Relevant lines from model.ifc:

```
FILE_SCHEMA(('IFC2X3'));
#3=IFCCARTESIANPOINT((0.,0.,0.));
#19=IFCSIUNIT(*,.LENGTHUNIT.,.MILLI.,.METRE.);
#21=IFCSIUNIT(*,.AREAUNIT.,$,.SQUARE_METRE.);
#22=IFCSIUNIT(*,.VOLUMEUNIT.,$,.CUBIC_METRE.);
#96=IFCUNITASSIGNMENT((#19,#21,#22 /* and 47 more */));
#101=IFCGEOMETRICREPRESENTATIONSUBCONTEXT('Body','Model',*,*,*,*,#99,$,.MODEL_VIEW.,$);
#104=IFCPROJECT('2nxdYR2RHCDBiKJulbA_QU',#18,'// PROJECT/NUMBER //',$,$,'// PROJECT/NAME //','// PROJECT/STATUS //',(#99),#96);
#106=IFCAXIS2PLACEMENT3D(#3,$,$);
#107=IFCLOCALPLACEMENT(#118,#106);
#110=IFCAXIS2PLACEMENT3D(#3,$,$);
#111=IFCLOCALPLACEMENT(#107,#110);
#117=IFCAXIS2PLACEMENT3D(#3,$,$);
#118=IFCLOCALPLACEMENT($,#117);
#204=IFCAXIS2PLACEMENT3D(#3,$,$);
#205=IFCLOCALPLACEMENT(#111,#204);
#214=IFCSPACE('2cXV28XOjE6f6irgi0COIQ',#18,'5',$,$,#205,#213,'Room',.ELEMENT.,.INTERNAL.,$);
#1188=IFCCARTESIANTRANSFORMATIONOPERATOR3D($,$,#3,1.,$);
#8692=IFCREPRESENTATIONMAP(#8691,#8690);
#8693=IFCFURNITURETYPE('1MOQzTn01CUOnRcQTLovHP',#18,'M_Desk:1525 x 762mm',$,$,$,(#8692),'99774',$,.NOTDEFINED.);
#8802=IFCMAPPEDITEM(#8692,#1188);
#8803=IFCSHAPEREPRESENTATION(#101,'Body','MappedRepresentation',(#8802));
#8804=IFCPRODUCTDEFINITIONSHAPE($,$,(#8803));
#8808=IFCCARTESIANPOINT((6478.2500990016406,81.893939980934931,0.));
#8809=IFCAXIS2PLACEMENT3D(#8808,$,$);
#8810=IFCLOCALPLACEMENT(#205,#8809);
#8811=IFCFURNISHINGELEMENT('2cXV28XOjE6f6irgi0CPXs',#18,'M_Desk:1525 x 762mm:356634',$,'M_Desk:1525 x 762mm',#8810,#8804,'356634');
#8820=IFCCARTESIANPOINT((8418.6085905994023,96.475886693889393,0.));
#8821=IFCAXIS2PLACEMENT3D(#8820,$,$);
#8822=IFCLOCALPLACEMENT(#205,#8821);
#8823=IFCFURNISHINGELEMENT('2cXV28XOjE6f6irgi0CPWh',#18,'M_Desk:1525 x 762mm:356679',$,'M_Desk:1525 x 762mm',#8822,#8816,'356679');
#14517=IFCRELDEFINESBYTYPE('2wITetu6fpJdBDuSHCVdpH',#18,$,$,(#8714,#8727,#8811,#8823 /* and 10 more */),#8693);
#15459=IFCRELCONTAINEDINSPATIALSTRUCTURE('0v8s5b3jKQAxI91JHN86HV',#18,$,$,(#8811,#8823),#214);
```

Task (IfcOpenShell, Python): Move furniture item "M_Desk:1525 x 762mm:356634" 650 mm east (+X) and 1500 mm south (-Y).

```python
import ifcopenshell
import ifcopenshell.api.geometry
import ifcopenshell.util.placement
import ifcopenshell.util.unit

model = ifcopenshell.open("model.ifc")
unit_scale = ifcopenshell.util.unit.calculate_unit_scale(model)

item = model.by_guid("2cXV28XOjE6f6irgi0CPXs")
matrix = ifcopenshell.util.placement.get_local_placement(item.ObjectPlacement)
matrix[0, 3] += 0.65 / unit_scale
matrix[1, 3] -= 1.5 / unit_scale
ifcopenshell.api.geometry.edit_object_placement(model, product=item, matrix=matrix, is_si=False)

print(ifcopenshell.util.placement.get_local_placement(item.ObjectPlacement).round(3) + 0.0)

model.write("model_v2.ifc")
```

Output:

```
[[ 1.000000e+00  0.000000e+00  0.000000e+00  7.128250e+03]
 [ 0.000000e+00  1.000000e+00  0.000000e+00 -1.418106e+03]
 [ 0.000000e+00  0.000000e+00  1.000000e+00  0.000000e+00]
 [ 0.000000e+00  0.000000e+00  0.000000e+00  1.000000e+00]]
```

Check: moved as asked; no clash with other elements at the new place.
